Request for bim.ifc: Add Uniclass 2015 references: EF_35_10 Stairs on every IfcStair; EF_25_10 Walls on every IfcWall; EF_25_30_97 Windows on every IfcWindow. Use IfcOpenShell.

First a look at what the model holds.

```python
import ifcopenshell

model = ifcopenshell.open("bim.ifc")
print(model.schema)
print("classifications:", [c.Name for c in model.by_type("IfcClassification")])
for ifc_class in ("IfcDoor", "IfcRoof", "IfcStair", "IfcWall", "IfcWindow"):
    print(ifc_class, len(model.by_type(ifc_class)))
```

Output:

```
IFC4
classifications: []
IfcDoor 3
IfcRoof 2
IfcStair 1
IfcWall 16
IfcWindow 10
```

```python
import ifcopenshell
import ifcopenshell.api.classification

model = ifcopenshell.open("bim.ifc")

system = ifcopenshell.api.classification.add_classification(model, classification="Uniclass 2015")

codes = {
    "IfcStair": ("EF_35_10", "Stairs"),
    "IfcWall": ("EF_25_10", "Walls"),
    "IfcWindow": ("EF_25_30_97", "Windows"),
}
for ifc_class, (code, name) in codes.items():
    products = model.by_type(ifc_class)
    ifcopenshell.api.classification.add_reference(
        model, products=products, classification=system, identification=code, name=name
    )
    print(code, len(products))

model.write("bim_rev.ifc")
```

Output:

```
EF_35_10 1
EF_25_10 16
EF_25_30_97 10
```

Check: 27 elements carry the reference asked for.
